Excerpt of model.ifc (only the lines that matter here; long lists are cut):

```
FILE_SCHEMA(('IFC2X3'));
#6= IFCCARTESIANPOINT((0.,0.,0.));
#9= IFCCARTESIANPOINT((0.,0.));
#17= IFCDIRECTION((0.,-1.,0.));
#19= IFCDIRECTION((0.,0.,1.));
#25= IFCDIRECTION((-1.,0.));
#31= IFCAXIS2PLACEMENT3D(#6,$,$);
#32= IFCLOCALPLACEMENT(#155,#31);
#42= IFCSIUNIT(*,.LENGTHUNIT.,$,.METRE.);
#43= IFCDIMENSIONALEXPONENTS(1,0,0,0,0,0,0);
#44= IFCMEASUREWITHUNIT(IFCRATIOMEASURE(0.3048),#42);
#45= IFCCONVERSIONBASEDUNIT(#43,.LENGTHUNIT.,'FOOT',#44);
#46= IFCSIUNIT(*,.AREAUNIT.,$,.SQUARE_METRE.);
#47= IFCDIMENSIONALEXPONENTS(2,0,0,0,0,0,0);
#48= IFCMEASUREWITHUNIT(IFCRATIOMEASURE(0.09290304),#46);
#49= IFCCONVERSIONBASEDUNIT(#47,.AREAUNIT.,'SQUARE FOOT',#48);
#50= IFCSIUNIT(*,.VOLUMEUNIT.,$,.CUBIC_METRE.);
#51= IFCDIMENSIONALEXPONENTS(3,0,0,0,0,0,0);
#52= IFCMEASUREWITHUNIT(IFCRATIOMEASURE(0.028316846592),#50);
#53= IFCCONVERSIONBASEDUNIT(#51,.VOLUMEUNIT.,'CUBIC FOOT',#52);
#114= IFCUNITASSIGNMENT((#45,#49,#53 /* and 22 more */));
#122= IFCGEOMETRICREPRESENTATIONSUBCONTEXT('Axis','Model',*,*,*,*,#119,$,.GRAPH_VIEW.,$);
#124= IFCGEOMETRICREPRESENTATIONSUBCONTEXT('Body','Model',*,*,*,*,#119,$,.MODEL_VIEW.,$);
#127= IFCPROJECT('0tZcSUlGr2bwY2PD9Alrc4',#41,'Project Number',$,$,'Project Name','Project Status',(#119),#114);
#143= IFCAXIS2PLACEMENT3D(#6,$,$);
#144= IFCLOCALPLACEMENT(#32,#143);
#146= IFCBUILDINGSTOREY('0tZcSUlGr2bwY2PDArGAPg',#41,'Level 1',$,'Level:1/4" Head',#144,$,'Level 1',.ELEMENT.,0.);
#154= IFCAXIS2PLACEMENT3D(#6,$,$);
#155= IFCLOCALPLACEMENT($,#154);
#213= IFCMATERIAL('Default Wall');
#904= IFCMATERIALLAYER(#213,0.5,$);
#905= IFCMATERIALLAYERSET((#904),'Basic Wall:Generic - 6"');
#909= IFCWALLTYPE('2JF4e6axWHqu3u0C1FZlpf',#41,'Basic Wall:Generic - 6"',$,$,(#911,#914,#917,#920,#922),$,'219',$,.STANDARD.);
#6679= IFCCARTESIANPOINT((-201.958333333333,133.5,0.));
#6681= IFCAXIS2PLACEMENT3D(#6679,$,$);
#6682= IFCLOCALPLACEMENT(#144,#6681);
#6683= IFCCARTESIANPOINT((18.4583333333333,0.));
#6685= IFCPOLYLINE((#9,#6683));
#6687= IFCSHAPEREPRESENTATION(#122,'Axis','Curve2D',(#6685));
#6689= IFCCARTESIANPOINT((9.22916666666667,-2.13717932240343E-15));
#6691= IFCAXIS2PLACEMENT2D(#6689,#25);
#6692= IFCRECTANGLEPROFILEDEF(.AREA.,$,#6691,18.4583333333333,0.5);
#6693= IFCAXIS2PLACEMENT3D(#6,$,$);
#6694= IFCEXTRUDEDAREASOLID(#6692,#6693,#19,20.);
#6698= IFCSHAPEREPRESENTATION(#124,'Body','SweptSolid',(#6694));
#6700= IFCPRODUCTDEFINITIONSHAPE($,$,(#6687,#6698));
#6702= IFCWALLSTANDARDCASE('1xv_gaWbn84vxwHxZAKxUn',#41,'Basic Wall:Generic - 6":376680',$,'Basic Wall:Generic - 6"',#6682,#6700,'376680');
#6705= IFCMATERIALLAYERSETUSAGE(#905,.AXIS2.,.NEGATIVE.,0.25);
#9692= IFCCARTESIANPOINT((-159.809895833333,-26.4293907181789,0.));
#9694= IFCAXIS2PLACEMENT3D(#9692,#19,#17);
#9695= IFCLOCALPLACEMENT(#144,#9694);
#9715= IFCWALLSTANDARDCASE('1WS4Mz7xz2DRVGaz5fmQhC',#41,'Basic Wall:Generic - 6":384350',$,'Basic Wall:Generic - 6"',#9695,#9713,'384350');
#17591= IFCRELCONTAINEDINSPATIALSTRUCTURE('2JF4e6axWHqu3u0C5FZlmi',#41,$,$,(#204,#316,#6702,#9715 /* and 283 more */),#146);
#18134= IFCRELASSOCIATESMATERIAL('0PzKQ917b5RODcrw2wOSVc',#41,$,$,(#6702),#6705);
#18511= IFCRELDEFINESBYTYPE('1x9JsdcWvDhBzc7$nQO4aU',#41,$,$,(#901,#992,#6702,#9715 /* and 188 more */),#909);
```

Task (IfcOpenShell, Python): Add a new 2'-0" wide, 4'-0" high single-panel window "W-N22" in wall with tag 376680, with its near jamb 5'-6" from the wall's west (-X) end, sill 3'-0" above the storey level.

```python
import numpy as np
import ifcopenshell
import ifcopenshell.api.feature
import ifcopenshell.api.geometry
import ifcopenshell.api.root
import ifcopenshell.api.spatial
import ifcopenshell.api.type
import ifcopenshell.geom
import ifcopenshell.util.element
import ifcopenshell.util.placement
import ifcopenshell.util.representation
import ifcopenshell.util.shape
import ifcopenshell.util.unit

model = ifcopenshell.open("model.ifc")
unit_scale = ifcopenshell.util.unit.calculate_unit_scale(model)
settings = ifcopenshell.geom.settings()


def volume(element):
    """Net volume in cubic metres, openings subtracted."""
    shape = ifcopenshell.geom.create_shape(settings, element)
    return ifcopenshell.util.shape.get_volume(shape.geometry)


wall = model.by_guid("1xv_gaWbn84vxwHxZAKxUn")
storey = ifcopenshell.util.element.get_container(wall, ifc_class="IfcBuildingStorey")
context = ifcopenshell.util.representation.get_context(model, "Model", "Body", "MODEL_VIEW")
before = volume(wall)

width, height, from_end, sill = 0.6096, 1.2192, 1.6764, 0.9144  # metres

# The wall runs along its own X axis, and the end named is its -X end.
wall_shape = ifcopenshell.geom.create_shape(settings, wall)
x, y, z = ifcopenshell.util.shape.get_vertices(wall_shape.geometry).T
start = x.min() + from_end
face, thickness = float(y.min()), float(y.max() - y.min())
wall_matrix = ifcopenshell.util.placement.get_local_placement(wall.ObjectPlacement)
level = ifcopenshell.util.placement.get_local_placement(storey.ObjectPlacement)[2, 3]


def in_wall(x, y):
    """Placement at x, y metres in the wall's axes, at sill height."""
    matrix = wall_matrix.copy()
    matrix[:, 3] = wall_matrix @ np.array([x / unit_scale, y / unit_scale, 0.0, 1.0])
    matrix[2, 3] = level + sill / unit_scale
    return matrix


# Opening: a box that overshoots both wall faces by 50 mm.
opening = ifcopenshell.api.root.create_entity(model, ifc_class="IfcOpeningElement")
box = ifcopenshell.api.geometry.add_wall_representation(
    model, context=context, length=width, height=height, thickness=thickness + 0.1
)
ifcopenshell.api.geometry.assign_representation(model, product=opening, representation=box)
ifcopenshell.api.geometry.edit_object_placement(model, product=opening, matrix=in_wall(start, face - 0.05), is_si=False)
ifcopenshell.api.feature.add_feature(model, feature=opening, element=wall)

window = ifcopenshell.api.root.create_entity(model, ifc_class="IfcWindow", name="W-N22")
window.OverallWidth, window.OverallHeight = width / unit_scale, height / unit_scale
body = ifcopenshell.api.geometry.add_window_representation(
    model,
    context=context,
    overall_width=window.OverallWidth,
    overall_height=window.OverallHeight,
    partition_type="SINGLE_PANEL",
)
ifcopenshell.api.geometry.assign_representation(model, product=window, representation=body)
ifcopenshell.api.spatial.assign_container(model, products=[window], relating_structure=storey)
fills = ifcopenshell.api.feature.add_filling(model, opening=opening, element=window)
fills.OwnerHistory = window.OwnerHistory  # required in IFC2X3

# IFC2X3 keeps the operation on the window style.
style = ifcopenshell.api.root.create_entity(model, ifc_class="IfcWindowStyle", name="W-N22")
style.OperationType, style.ConstructionType = "SINGLE_PANEL", "NOTDEFINED"
style.ParameterTakesPrecedence = style.Sizeable = False
ifcopenshell.api.type.assign_type(model, related_objects=[window], relating_type=style)

# Centre the window in the wall's thickness.
ifcopenshell.api.geometry.edit_object_placement(model, product=window, matrix=in_wall(start, face), is_si=False)
window_shape = ifcopenshell.geom.create_shape(settings, window)
depth = ifcopenshell.util.shape.get_vertices(window_shape.geometry)[:, 1]
offset = face + thickness / 2 - (depth.min() + depth.max()) / 2
ifcopenshell.api.geometry.edit_object_placement(model, product=window, matrix=in_wall(start, offset), is_si=False)

after = volume(wall)

print(f"wall volume {before:.3f} -> {after:.3f} m3")

model.write("model_rev.ifc")
```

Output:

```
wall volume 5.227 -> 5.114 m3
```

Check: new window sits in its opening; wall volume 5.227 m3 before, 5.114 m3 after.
